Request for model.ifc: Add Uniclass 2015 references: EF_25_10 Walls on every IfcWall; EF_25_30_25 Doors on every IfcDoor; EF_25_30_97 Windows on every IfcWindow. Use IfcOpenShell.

First a look at what the model holds.

```python
import ifcopenshell

model = ifcopenshell.open("model.ifc")
print(model.schema)
print("classifications:", [c.Name for c in model.by_type("IfcClassification")])
for ifc_class in ("IfcDoor", "IfcRoof", "IfcStair", "IfcWall", "IfcWindow"):
    print(ifc_class, len(model.by_type(ifc_class)))
```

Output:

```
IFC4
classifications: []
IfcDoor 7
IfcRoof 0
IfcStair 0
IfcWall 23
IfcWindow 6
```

```python
import ifcopenshell
import ifcopenshell.api.classification

model = ifcopenshell.open("model.ifc")

system = ifcopenshell.api.classification.add_classification(model, classification="Uniclass 2015")

codes = {
    "IfcWall": ("EF_25_10", "Walls"),
    "IfcDoor": ("EF_25_30_25", "Doors"),
    "IfcWindow": ("EF_25_30_97", "Windows"),
}
for ifc_class, (code, name) in codes.items():
    products = model.by_type(ifc_class)
    ifcopenshell.api.classification.add_reference(
        model, products=products, classification=system, identification=code, name=name
    )
    print(code, len(products))

model.write("model_edited.ifc")
```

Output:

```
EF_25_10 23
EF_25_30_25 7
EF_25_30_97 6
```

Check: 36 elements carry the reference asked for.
